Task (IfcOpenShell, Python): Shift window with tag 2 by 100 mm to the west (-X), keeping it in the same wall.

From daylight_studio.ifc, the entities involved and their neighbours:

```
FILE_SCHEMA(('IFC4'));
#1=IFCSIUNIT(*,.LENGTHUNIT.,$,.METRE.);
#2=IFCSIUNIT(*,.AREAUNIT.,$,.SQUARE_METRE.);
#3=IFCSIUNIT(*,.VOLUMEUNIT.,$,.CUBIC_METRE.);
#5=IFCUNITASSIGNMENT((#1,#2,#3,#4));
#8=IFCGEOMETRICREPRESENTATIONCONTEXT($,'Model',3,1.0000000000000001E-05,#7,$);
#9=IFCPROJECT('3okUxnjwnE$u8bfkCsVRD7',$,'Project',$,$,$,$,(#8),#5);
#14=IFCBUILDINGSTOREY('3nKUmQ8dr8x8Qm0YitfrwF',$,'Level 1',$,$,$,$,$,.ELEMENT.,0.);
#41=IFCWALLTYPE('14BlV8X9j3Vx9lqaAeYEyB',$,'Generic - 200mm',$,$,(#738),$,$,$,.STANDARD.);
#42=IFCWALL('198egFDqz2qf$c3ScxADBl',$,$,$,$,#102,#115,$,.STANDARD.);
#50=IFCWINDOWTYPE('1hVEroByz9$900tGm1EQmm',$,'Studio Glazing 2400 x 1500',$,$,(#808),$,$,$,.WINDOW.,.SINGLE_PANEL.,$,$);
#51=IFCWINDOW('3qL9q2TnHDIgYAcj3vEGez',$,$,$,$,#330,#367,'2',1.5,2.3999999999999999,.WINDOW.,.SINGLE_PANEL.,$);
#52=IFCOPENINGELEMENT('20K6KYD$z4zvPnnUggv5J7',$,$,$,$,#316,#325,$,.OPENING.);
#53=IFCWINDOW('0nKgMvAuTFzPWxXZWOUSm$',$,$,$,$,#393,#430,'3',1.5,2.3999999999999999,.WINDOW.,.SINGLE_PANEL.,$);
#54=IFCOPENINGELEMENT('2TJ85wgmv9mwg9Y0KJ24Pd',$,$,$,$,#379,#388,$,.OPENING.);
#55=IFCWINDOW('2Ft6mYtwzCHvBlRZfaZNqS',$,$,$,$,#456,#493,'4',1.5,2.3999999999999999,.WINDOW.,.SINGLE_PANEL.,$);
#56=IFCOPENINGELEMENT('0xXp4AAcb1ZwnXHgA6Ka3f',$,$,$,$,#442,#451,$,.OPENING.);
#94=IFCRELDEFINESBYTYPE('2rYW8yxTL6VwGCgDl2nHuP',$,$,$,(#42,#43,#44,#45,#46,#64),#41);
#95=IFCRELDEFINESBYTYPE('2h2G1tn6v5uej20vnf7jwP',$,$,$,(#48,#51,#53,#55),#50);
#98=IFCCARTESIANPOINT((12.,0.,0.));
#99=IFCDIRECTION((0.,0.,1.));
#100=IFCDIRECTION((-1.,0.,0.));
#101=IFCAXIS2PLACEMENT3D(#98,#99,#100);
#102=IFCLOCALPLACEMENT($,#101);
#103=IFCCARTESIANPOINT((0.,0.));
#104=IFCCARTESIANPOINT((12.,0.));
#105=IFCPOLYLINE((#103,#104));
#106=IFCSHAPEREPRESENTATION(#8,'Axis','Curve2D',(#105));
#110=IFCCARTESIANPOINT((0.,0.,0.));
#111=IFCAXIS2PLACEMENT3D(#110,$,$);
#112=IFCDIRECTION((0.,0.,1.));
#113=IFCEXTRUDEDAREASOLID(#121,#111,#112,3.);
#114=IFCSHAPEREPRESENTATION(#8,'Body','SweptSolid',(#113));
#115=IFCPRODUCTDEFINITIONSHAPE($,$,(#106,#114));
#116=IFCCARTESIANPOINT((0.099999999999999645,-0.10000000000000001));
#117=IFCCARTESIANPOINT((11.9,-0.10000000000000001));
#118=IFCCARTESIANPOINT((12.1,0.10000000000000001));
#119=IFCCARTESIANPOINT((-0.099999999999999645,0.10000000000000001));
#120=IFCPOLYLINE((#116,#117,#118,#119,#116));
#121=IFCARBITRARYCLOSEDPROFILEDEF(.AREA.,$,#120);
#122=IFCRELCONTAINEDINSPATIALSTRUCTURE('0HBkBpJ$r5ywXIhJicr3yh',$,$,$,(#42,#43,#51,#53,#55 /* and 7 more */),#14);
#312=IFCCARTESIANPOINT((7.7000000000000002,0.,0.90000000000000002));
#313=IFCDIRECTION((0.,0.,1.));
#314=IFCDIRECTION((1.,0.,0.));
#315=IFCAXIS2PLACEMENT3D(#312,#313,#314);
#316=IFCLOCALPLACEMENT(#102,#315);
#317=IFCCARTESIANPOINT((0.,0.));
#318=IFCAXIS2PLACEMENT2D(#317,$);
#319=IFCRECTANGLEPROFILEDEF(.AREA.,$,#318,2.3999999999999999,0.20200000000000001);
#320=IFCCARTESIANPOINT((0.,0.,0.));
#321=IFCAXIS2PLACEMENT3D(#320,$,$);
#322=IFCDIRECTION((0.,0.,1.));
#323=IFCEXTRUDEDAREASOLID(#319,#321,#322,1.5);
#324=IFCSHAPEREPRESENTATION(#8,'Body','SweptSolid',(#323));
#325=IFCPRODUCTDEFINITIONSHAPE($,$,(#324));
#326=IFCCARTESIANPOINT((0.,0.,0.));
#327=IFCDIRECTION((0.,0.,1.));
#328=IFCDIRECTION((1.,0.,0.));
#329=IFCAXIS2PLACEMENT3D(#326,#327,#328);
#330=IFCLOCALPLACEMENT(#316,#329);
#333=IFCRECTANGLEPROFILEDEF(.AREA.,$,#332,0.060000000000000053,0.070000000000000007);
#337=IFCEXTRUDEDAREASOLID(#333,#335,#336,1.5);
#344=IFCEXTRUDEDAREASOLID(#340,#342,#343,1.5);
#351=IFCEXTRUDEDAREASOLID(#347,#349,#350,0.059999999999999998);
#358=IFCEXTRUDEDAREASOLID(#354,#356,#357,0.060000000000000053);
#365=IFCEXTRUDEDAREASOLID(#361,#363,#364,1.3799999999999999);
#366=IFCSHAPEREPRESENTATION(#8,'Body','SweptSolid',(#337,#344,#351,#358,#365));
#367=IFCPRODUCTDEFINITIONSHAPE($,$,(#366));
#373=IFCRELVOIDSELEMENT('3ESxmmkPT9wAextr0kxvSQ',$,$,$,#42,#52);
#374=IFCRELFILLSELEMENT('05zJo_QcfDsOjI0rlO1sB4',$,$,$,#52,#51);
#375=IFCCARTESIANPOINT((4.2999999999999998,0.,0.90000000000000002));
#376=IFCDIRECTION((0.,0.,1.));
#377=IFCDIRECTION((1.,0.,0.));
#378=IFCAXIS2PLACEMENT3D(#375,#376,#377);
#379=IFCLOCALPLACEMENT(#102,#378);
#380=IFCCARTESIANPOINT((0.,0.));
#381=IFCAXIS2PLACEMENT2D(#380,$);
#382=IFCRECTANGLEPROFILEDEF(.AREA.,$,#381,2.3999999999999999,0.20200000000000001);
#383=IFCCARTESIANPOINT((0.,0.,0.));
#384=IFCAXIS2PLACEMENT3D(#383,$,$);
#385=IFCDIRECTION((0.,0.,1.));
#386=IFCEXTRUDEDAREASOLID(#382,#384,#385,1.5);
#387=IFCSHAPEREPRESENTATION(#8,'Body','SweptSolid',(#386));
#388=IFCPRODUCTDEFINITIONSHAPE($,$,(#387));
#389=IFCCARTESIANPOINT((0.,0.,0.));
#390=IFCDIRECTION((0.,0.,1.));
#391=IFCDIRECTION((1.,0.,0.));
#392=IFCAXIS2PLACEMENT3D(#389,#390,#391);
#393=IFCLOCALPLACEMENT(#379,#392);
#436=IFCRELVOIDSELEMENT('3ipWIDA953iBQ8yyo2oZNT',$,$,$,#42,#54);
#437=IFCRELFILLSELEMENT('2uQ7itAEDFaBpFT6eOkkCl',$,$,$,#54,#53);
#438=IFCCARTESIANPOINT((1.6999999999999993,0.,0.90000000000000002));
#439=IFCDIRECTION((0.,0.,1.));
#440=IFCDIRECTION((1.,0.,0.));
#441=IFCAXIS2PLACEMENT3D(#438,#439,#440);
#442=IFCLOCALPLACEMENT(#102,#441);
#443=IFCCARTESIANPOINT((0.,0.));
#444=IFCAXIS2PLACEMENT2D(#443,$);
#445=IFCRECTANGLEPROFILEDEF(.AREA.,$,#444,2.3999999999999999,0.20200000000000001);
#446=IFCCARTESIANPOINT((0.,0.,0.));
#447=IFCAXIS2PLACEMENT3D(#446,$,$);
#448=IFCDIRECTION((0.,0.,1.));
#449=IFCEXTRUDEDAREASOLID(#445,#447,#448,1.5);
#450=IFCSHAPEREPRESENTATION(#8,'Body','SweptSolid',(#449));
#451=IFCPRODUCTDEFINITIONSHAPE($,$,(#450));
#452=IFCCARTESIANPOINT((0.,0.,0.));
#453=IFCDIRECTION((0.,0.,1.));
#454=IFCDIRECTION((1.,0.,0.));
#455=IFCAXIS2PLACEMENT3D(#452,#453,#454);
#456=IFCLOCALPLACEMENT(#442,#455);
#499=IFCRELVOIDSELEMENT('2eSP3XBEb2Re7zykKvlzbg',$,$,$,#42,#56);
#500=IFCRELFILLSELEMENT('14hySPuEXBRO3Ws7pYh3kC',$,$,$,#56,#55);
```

```python
import ifcopenshell
import ifcopenshell.api.geometry
import ifcopenshell.util.placement
import ifcopenshell.util.unit

model = ifcopenshell.open("daylight_studio.ifc")
unit_scale = ifcopenshell.util.unit.calculate_unit_scale(model)

window = model.by_guid("3qL9q2TnHDIgYAcj3vEGez")
opening = window.FillsVoids[0].RelatingOpeningElement
wall = opening.VoidsElements[0].RelatingBuildingElement

wall_matrix = ifcopenshell.util.placement.get_local_placement(wall.ObjectPlacement)
shift = wall_matrix[:3, 0] * 0.1 / unit_scale
before = ifcopenshell.util.placement.get_local_placement(window.ObjectPlacement)[:3, 3].copy()

# The window is placed relative to its opening, so it follows when the opening moves.
matrix = ifcopenshell.util.placement.get_local_placement(opening.ObjectPlacement)
matrix[:3, 3] += shift
ifcopenshell.api.geometry.edit_object_placement(
    model, product=opening, matrix=matrix, is_si=False, should_transform_children=True
)

after = ifcopenshell.util.placement.get_local_placement(window.ObjectPlacement)[:3, 3]
print("window moved by", (after - before).round(3) + 0.0)

model.write("daylight_studio_rev.ifc")
```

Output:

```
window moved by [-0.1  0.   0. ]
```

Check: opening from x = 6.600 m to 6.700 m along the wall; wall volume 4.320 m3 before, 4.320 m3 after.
